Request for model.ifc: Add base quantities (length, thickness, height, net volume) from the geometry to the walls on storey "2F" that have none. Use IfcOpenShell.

First a look at what the model holds.

```python
import ifcopenshell
import ifcopenshell.util.element
import ifcopenshell.util.unit

model = ifcopenshell.open("model.ifc")
print(model.schema)
for unit_type in ("LENGTHUNIT", "AREAUNIT", "VOLUMEUNIT"):
    print(unit_type, ifcopenshell.util.unit.calculate_unit_scale(model, unit_type))
storey = next(s for s in model.by_type("IfcBuildingStorey") if s.Name == "2F")
walls = [e for e in ifcopenshell.util.element.get_decomposition(storey) if e.is_a("IfcWall")]
for e in sorted(walls, key=lambda e: e.id()):
    print(e.id(), e.is_a(), e.Name, list(ifcopenshell.util.element.get_psets(e, qtos_only=True)), sep=" | ")
```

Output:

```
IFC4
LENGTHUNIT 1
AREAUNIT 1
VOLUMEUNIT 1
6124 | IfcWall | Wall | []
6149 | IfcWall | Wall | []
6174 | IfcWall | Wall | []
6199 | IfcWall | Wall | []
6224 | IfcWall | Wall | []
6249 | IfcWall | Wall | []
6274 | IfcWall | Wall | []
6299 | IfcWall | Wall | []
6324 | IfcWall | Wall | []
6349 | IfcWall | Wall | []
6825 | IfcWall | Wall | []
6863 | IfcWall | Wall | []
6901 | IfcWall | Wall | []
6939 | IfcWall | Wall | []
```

```python
import ifcopenshell
import ifcopenshell.api.pset
import ifcopenshell.geom
import ifcopenshell.util.element
import ifcopenshell.util.shape
import ifcopenshell.util.unit

model = ifcopenshell.open("model.ifc")
unit_scale = ifcopenshell.util.unit.calculate_unit_scale(model)
volume_scale = ifcopenshell.util.unit.calculate_unit_scale(model, "VOLUMEUNIT")
settings = ifcopenshell.geom.settings()

storey = next(s for s in model.by_type("IfcBuildingStorey") if s.Name == "2F")
walls = [e for e in ifcopenshell.util.element.get_decomposition(storey) if e.is_a("IfcWall")]

for e in sorted(walls, key=lambda e: e.id()):
    if ifcopenshell.util.element.get_psets(e, qtos_only=True, should_inherit=False):
        continue
    # Geometry comes back in metres, in the element's own axes.
    shape = ifcopenshell.geom.create_shape(settings, e)
    values = {
        "Length": ifcopenshell.util.shape.get_x(shape.geometry) / unit_scale,
        "Width": ifcopenshell.util.shape.get_y(shape.geometry) / unit_scale,
        "Height": ifcopenshell.util.shape.get_z(shape.geometry) / unit_scale,
        "NetVolume": ifcopenshell.util.shape.get_volume(shape.geometry) / volume_scale,
    }
    qto = ifcopenshell.api.pset.add_qto(model, product=e, name="Qto_WallBaseQuantities")
    ifcopenshell.api.pset.edit_qto(model, qto=qto, properties=values)
    print(e.id(), {k: round(v, 3) for k, v in values.items()})

model.write("model_edited.ifc")
```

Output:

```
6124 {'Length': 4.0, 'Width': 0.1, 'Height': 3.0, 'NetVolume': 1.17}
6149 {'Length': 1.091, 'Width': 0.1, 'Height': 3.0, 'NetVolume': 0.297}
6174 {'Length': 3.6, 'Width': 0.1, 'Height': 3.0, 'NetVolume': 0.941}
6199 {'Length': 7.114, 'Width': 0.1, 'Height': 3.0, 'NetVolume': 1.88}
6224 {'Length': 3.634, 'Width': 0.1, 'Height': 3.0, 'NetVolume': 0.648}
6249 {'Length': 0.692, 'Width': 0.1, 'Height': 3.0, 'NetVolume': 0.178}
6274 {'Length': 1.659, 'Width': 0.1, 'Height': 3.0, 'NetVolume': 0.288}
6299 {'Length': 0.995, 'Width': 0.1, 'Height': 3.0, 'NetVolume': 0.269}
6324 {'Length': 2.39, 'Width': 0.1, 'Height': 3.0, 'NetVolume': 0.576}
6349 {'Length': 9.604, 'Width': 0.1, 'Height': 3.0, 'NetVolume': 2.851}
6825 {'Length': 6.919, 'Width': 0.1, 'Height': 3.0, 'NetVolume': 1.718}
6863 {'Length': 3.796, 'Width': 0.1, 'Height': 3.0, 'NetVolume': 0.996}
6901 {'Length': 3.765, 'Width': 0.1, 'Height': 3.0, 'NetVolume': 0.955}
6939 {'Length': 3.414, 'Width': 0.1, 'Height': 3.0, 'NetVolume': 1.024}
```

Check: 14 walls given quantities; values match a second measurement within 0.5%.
